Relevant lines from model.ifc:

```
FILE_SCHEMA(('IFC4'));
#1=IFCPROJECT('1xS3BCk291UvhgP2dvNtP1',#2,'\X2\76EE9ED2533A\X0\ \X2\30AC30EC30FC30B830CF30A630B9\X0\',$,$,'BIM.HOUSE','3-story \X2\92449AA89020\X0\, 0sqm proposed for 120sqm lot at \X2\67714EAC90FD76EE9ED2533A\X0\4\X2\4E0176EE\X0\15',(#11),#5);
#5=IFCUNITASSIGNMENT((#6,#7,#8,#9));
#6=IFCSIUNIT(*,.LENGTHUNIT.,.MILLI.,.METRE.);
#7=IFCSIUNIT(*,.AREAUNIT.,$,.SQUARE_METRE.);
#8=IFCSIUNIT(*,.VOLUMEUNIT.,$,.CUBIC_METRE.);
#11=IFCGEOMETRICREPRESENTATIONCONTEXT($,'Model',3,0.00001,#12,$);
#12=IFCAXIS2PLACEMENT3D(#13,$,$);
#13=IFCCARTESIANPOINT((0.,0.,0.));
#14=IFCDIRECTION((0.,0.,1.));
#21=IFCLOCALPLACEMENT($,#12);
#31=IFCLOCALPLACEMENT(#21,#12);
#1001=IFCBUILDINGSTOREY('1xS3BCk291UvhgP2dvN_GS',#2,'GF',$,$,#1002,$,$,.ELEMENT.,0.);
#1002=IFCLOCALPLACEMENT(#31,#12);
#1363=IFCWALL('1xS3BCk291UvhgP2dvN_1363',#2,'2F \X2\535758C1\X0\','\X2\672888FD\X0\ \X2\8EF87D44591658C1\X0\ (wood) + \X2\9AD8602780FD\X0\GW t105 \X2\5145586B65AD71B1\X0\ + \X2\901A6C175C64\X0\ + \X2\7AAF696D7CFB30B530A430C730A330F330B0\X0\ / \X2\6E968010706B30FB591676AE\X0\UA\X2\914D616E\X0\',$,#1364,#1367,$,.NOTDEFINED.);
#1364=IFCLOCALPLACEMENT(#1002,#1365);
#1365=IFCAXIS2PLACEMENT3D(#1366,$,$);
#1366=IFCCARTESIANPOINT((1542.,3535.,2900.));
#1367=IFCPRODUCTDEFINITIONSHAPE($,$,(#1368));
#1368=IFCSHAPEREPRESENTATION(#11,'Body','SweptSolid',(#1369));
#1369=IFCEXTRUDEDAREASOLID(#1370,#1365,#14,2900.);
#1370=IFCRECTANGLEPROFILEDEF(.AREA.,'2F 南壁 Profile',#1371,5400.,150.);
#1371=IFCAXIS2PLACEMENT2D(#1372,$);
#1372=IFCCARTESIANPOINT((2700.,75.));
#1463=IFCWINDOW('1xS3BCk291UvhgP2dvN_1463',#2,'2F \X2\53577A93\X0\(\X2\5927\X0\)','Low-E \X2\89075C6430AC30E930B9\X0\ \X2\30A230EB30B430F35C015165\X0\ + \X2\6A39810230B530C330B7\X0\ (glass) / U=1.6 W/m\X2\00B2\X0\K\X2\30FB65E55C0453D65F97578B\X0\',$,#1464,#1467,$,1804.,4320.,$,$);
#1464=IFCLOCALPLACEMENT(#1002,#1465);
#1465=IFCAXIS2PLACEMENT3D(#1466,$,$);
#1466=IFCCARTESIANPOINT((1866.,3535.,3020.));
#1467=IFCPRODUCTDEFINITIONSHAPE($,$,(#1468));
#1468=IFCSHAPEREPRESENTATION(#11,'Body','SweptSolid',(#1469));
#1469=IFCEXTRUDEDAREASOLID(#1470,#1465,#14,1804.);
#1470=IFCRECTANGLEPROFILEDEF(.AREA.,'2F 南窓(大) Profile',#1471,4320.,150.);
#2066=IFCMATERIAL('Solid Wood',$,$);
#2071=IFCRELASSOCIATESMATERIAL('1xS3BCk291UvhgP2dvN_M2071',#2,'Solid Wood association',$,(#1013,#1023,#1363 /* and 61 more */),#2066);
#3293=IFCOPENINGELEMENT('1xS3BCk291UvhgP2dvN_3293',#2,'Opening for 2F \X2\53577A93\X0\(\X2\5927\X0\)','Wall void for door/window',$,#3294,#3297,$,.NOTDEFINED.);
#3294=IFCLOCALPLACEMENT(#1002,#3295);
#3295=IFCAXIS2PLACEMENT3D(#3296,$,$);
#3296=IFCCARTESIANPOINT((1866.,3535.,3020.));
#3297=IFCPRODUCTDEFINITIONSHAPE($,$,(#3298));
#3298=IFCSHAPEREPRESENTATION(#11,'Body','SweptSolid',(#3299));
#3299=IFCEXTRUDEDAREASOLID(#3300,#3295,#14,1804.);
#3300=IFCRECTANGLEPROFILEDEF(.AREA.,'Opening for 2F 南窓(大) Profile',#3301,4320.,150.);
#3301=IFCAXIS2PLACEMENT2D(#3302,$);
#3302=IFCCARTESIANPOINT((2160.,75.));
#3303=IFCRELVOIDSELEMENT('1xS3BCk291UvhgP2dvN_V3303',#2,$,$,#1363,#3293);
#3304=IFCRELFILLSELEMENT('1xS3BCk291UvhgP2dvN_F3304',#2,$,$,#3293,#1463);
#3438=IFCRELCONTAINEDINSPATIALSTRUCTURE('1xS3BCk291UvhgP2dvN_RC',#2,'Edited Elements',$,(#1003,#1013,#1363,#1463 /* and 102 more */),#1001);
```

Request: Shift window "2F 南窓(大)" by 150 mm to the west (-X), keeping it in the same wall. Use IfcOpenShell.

```python
import ifcopenshell
import ifcopenshell.api.geometry
import ifcopenshell.util.placement
import ifcopenshell.util.unit

model = ifcopenshell.open("model.ifc")
unit_scale = ifcopenshell.util.unit.calculate_unit_scale(model)

window = model.by_guid("1xS3BCk291UvhgP2dvN_1463")
opening = window.FillsVoids[0].RelatingOpeningElement
wall = opening.VoidsElements[0].RelatingBuildingElement

wall_matrix = ifcopenshell.util.placement.get_local_placement(wall.ObjectPlacement)
shift = wall_matrix[:3, 0] * -0.15 / unit_scale
before = ifcopenshell.util.placement.get_local_placement(window.ObjectPlacement)[:3, 3].copy()

# The window is not placed relative to its opening, so move both.
for product in (opening, window):
    matrix = ifcopenshell.util.placement.get_local_placement(product.ObjectPlacement)
    matrix[:3, 3] += shift
    ifcopenshell.api.geometry.edit_object_placement(model, product=product, matrix=matrix, is_si=False)

after = ifcopenshell.util.placement.get_local_placement(window.ObjectPlacement)[:3, 3]
print("window moved by", (after - before).round(3) + 0.0)

model.write("model_updated.ifc")
```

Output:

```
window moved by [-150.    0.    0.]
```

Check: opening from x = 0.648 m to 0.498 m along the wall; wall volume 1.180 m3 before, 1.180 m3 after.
